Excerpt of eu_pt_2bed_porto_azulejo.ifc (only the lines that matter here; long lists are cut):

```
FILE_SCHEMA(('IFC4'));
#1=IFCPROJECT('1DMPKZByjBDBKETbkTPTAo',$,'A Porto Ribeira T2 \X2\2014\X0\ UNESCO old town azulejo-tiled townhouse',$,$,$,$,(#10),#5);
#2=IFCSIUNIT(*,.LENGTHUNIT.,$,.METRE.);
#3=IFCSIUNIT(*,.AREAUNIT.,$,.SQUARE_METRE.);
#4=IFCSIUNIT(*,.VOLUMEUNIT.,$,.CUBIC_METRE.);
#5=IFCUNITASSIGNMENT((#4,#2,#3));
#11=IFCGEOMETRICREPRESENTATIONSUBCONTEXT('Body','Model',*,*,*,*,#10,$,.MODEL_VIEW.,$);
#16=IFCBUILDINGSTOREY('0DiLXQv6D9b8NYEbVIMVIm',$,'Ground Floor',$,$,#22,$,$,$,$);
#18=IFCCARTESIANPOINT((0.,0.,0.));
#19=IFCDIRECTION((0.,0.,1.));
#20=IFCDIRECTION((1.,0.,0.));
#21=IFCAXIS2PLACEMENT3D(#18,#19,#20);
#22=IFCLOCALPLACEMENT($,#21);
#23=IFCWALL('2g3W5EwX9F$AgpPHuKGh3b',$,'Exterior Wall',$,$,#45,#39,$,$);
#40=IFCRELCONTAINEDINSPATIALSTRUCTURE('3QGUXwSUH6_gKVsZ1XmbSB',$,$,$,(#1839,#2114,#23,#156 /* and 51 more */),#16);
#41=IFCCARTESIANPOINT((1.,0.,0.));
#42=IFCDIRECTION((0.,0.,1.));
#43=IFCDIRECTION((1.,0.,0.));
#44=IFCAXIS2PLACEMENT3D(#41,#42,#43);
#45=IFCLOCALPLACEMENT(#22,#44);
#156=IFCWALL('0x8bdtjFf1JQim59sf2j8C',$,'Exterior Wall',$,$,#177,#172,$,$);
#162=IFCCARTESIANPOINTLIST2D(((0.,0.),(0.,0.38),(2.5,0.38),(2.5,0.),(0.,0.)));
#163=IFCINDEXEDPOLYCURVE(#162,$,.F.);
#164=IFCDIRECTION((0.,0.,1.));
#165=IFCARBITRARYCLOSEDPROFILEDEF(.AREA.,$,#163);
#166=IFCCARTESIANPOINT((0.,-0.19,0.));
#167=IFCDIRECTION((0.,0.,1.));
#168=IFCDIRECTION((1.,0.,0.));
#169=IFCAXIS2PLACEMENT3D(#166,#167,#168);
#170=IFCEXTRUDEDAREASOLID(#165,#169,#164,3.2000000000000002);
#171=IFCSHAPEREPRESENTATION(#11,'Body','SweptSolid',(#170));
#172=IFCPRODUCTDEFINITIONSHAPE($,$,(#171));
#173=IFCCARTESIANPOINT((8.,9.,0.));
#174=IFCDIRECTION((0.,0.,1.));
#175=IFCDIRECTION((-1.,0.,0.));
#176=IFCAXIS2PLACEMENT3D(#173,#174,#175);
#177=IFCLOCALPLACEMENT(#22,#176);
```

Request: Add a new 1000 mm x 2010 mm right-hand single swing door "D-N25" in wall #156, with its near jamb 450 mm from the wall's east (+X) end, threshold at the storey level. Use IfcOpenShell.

```python
import numpy as np
import ifcopenshell
import ifcopenshell.api.feature
import ifcopenshell.api.geometry
import ifcopenshell.api.root
import ifcopenshell.api.spatial
import ifcopenshell.geom
import ifcopenshell.util.element
import ifcopenshell.util.placement
import ifcopenshell.util.representation
import ifcopenshell.util.shape
import ifcopenshell.util.unit

model = ifcopenshell.open("eu_pt_2bed_porto_azulejo.ifc")
unit_scale = ifcopenshell.util.unit.calculate_unit_scale(model)
settings = ifcopenshell.geom.settings()


def volume(element):
    """Net volume in cubic metres, openings subtracted."""
    shape = ifcopenshell.geom.create_shape(settings, element)
    return ifcopenshell.util.shape.get_volume(shape.geometry)


wall = model.by_guid("0x8bdtjFf1JQim59sf2j8C")
storey = ifcopenshell.util.element.get_container(wall, ifc_class="IfcBuildingStorey")
context = ifcopenshell.util.representation.get_context(model, "Model", "Body", "MODEL_VIEW")
before = volume(wall)

width, height, from_end, sill = 1, 2.01, 0.45, 0.0  # metres

# The wall runs along its own X axis, and the end named is its -X end.
wall_shape = ifcopenshell.geom.create_shape(settings, wall)
x, y, z = ifcopenshell.util.shape.get_vertices(wall_shape.geometry).T
start = x.min() + from_end
face, thickness = float(y.min()), float(y.max() - y.min())
wall_matrix = ifcopenshell.util.placement.get_local_placement(wall.ObjectPlacement)
level = ifcopenshell.util.placement.get_local_placement(storey.ObjectPlacement)[2, 3]


def in_wall(x, y):
    """Placement at x, y metres in the wall's axes, at sill height."""
    matrix = wall_matrix.copy()
    matrix[:, 3] = wall_matrix @ np.array([x / unit_scale, y / unit_scale, 0.0, 1.0])
    matrix[2, 3] = level + sill / unit_scale
    return matrix


# Opening: a box that overshoots both wall faces by 50 mm.
opening = ifcopenshell.api.root.create_entity(model, ifc_class="IfcOpeningElement", predefined_type="OPENING")
box = ifcopenshell.api.geometry.add_wall_representation(
    model, context=context, length=width, height=height, thickness=thickness + 0.1
)
ifcopenshell.api.geometry.assign_representation(model, product=opening, representation=box)
ifcopenshell.api.geometry.edit_object_placement(model, product=opening, matrix=in_wall(start, face - 0.05), is_si=False)
ifcopenshell.api.feature.add_feature(model, feature=opening, element=wall)

door = ifcopenshell.api.root.create_entity(model, ifc_class="IfcDoor", name="D-N25", predefined_type="DOOR")
door.OverallWidth, door.OverallHeight = width / unit_scale, height / unit_scale
door.OperationType = "SINGLE_SWING_RIGHT"
body = ifcopenshell.api.geometry.add_door_representation(
    model,
    context=context,
    overall_width=door.OverallWidth,
    overall_height=door.OverallHeight,
    operation_type="SINGLE_SWING_RIGHT",
    lining_properties={"LiningDepth": thickness / unit_scale, "ThresholdDepth": thickness / unit_scale},
)
ifcopenshell.api.geometry.assign_representation(model, product=door, representation=body)
ifcopenshell.api.spatial.assign_container(model, products=[door], relating_structure=storey)
ifcopenshell.api.feature.add_filling(model, opening=opening, element=door)

# The lining spans the wall, so the door starts at the wall face.
ifcopenshell.api.geometry.edit_object_placement(model, product=door, matrix=in_wall(start, face), is_si=False)

after = volume(wall)

print(f"wall volume {before:.3f} -> {after:.3f} m3")

model.write("eu_pt_2bed_porto_azulejo_v2.ifc")
```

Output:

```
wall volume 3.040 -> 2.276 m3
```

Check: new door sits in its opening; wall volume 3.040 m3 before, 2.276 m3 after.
